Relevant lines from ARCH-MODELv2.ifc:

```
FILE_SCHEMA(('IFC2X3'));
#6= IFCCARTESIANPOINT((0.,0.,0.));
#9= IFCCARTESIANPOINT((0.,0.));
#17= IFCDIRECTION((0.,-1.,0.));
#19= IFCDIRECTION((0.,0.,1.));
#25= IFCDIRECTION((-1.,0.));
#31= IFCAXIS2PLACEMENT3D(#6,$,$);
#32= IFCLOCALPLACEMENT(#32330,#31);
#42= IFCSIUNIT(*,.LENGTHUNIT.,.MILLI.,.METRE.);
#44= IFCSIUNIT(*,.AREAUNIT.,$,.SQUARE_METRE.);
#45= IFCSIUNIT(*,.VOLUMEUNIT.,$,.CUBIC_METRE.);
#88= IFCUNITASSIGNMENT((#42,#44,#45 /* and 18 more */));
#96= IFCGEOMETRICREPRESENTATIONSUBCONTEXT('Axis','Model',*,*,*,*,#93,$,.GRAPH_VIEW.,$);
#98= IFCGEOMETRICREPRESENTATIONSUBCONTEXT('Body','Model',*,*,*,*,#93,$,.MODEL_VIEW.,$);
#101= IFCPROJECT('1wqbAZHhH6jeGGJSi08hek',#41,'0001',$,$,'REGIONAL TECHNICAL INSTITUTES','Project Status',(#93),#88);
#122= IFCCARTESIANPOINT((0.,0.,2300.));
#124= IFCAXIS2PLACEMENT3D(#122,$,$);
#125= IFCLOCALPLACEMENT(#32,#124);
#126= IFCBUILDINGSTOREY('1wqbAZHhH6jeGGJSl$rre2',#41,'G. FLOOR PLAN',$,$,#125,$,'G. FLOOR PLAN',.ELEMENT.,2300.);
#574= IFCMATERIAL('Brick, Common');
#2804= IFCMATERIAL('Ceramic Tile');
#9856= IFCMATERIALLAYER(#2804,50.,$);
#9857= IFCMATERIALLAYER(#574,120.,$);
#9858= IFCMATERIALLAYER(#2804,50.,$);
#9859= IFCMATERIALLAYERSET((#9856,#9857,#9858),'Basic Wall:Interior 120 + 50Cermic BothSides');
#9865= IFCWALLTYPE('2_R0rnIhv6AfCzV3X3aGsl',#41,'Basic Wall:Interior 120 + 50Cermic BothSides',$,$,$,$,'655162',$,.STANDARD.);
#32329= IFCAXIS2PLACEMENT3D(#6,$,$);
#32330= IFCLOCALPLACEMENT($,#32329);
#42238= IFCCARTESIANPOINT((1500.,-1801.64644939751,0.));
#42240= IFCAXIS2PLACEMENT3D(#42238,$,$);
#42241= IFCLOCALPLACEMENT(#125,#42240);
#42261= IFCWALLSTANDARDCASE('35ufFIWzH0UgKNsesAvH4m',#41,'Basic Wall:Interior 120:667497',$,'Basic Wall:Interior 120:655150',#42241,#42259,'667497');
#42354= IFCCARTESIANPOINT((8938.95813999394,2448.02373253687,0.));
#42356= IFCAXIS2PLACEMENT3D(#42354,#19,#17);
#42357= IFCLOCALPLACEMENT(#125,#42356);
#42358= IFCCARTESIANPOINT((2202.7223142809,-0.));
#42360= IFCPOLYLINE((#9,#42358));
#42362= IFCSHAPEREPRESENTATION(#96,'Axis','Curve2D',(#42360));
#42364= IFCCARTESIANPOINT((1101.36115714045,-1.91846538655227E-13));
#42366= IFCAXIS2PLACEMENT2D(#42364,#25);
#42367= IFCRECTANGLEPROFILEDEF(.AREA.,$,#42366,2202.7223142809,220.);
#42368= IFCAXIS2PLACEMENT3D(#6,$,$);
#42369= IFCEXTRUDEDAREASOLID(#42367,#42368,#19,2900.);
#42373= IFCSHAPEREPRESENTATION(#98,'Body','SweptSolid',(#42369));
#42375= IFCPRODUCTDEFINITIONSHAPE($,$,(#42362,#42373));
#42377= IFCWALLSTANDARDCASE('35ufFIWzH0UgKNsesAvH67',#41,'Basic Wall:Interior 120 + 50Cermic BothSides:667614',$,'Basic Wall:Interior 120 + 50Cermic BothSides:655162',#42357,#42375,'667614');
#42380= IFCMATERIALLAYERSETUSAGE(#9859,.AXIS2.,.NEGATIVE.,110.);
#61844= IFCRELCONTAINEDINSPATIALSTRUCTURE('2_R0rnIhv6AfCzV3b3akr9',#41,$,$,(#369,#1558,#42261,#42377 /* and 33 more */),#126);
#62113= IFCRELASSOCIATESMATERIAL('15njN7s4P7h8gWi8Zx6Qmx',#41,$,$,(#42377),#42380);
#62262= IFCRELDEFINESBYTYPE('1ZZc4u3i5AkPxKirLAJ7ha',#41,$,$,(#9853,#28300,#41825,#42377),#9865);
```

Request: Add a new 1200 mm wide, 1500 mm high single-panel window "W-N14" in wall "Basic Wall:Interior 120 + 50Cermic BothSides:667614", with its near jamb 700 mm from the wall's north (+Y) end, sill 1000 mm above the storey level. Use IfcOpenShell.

```python
import numpy as np
import ifcopenshell
import ifcopenshell.api.feature
import ifcopenshell.api.geometry
import ifcopenshell.api.root
import ifcopenshell.api.spatial
import ifcopenshell.api.type
import ifcopenshell.geom
import ifcopenshell.util.element
import ifcopenshell.util.placement
import ifcopenshell.util.representation
import ifcopenshell.util.shape
import ifcopenshell.util.unit

model = ifcopenshell.open("ARCH-MODELv2.ifc")
unit_scale = ifcopenshell.util.unit.calculate_unit_scale(model)
settings = ifcopenshell.geom.settings()


def volume(element):
    """Net volume in cubic metres, openings subtracted."""
    shape = ifcopenshell.geom.create_shape(settings, element)
    return ifcopenshell.util.shape.get_volume(shape.geometry)


wall = model.by_guid("35ufFIWzH0UgKNsesAvH67")
storey = ifcopenshell.util.element.get_container(wall, ifc_class="IfcBuildingStorey")
context = ifcopenshell.util.representation.get_context(model, "Model", "Body", "MODEL_VIEW")
before = volume(wall)

width, height, from_end, sill = 1.2, 1.5, 0.7, 1  # metres

# The wall runs along its own X axis, and the end named is its -X end.
wall_shape = ifcopenshell.geom.create_shape(settings, wall)
x, y, z = ifcopenshell.util.shape.get_vertices(wall_shape.geometry).T
start = x.min() + from_end
face, thickness = float(y.min()), float(y.max() - y.min())
wall_matrix = ifcopenshell.util.placement.get_local_placement(wall.ObjectPlacement)
level = ifcopenshell.util.placement.get_local_placement(storey.ObjectPlacement)[2, 3]


def in_wall(x, y):
    """Placement at x, y metres in the wall's axes, at sill height."""
    matrix = wall_matrix.copy()
    matrix[:, 3] = wall_matrix @ np.array([x / unit_scale, y / unit_scale, 0.0, 1.0])
    matrix[2, 3] = level + sill / unit_scale
    return matrix


# Opening: a box that overshoots both wall faces by 50 mm.
opening = ifcopenshell.api.root.create_entity(model, ifc_class="IfcOpeningElement")
box = ifcopenshell.api.geometry.add_wall_representation(
    model, context=context, length=width, height=height, thickness=thickness + 0.1
)
ifcopenshell.api.geometry.assign_representation(model, product=opening, representation=box)
ifcopenshell.api.geometry.edit_object_placement(model, product=opening, matrix=in_wall(start, face - 0.05), is_si=False)
ifcopenshell.api.feature.add_feature(model, feature=opening, element=wall)

window = ifcopenshell.api.root.create_entity(model, ifc_class="IfcWindow", name="W-N14")
window.OverallWidth, window.OverallHeight = width / unit_scale, height / unit_scale
body = ifcopenshell.api.geometry.add_window_representation(
    model,
    context=context,
    overall_width=window.OverallWidth,
    overall_height=window.OverallHeight,
    partition_type="SINGLE_PANEL",
)
ifcopenshell.api.geometry.assign_representation(model, product=window, representation=body)
ifcopenshell.api.spatial.assign_container(model, products=[window], relating_structure=storey)
fills = ifcopenshell.api.feature.add_filling(model, opening=opening, element=window)
fills.OwnerHistory = window.OwnerHistory  # required in IFC2X3

# IFC2X3 keeps the operation on the window style.
style = ifcopenshell.api.root.create_entity(model, ifc_class="IfcWindowStyle", name="W-N14")
style.OperationType, style.ConstructionType = "SINGLE_PANEL", "NOTDEFINED"
style.ParameterTakesPrecedence = style.Sizeable = False
ifcopenshell.api.type.assign_type(model, related_objects=[window], relating_type=style)

# Centre the window in the wall's thickness.
ifcopenshell.api.geometry.edit_object_placement(model, product=window, matrix=in_wall(start, face), is_si=False)
window_shape = ifcopenshell.geom.create_shape(settings, window)
depth = ifcopenshell.util.shape.get_vertices(window_shape.geometry)[:, 1]
offset = face + thickness / 2 - (depth.min() + depth.max()) / 2
ifcopenshell.api.geometry.edit_object_placement(model, product=window, matrix=in_wall(start, offset), is_si=False)

after = volume(wall)

print(f"wall volume {before:.3f} -> {after:.3f} m3")

model.write("ARCH-MODELv2-out.ifc")
```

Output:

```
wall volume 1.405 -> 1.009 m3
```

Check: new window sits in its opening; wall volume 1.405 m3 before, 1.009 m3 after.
